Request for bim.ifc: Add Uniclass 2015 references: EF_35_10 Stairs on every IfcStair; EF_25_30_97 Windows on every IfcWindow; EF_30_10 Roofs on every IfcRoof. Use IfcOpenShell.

First a look at what the model holds.

```python
import ifcopenshell

model = ifcopenshell.open("bim.ifc")
print(model.schema)
print("classifications:", [c.Name for c in model.by_type("IfcClassification")])
for ifc_class in ("IfcDoor", "IfcRoof", "IfcStair", "IfcWall", "IfcWindow"):
    print(ifc_class, len(model.by_type(ifc_class)))
```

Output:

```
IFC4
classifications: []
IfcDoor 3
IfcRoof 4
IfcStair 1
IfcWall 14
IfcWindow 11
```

```python
import ifcopenshell
import ifcopenshell.api.classification

model = ifcopenshell.open("bim.ifc")

system = ifcopenshell.api.classification.add_classification(model, classification="Uniclass 2015")

codes = {
    "IfcStair": ("EF_35_10", "Stairs"),
    "IfcWindow": ("EF_25_30_97", "Windows"),
    "IfcRoof": ("EF_30_10", "Roofs"),
}
for ifc_class, (code, name) in codes.items():
    products = model.by_type(ifc_class)
    ifcopenshell.api.classification.add_reference(
        model, products=products, classification=system, identification=code, name=name
    )
    print(code, len(products))

model.write("bim_updated.ifc")
```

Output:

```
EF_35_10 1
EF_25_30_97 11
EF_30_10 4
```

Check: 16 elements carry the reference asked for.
